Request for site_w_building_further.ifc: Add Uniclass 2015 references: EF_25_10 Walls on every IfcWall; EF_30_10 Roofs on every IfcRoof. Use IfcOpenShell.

First a look at what the model holds.

```python
import ifcopenshell

model = ifcopenshell.open("site_w_building_further.ifc")
print(model.schema)
print("classifications:", [c.Name for c in model.by_type("IfcClassification")])
for ifc_class in ("IfcDoor", "IfcRoof", "IfcStair", "IfcWall", "IfcWindow"):
    print(ifc_class, len(model.by_type(ifc_class)))
```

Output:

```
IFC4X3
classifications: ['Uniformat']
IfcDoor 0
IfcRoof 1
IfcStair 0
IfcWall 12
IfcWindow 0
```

```python
import ifcopenshell
import ifcopenshell.api.classification

model = ifcopenshell.open("site_w_building_further.ifc")

system = ifcopenshell.api.classification.add_classification(model, classification="Uniclass 2015")

codes = {
    "IfcWall": ("EF_25_10", "Walls"),
    "IfcRoof": ("EF_30_10", "Roofs"),
}
for ifc_class, (code, name) in codes.items():
    products = model.by_type(ifc_class)
    ifcopenshell.api.classification.add_reference(
        model, products=products, classification=system, identification=code, name=name
    )
    print(code, len(products))

model.write("site_w_building_further_updated.ifc")
```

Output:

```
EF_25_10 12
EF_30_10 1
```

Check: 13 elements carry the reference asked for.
